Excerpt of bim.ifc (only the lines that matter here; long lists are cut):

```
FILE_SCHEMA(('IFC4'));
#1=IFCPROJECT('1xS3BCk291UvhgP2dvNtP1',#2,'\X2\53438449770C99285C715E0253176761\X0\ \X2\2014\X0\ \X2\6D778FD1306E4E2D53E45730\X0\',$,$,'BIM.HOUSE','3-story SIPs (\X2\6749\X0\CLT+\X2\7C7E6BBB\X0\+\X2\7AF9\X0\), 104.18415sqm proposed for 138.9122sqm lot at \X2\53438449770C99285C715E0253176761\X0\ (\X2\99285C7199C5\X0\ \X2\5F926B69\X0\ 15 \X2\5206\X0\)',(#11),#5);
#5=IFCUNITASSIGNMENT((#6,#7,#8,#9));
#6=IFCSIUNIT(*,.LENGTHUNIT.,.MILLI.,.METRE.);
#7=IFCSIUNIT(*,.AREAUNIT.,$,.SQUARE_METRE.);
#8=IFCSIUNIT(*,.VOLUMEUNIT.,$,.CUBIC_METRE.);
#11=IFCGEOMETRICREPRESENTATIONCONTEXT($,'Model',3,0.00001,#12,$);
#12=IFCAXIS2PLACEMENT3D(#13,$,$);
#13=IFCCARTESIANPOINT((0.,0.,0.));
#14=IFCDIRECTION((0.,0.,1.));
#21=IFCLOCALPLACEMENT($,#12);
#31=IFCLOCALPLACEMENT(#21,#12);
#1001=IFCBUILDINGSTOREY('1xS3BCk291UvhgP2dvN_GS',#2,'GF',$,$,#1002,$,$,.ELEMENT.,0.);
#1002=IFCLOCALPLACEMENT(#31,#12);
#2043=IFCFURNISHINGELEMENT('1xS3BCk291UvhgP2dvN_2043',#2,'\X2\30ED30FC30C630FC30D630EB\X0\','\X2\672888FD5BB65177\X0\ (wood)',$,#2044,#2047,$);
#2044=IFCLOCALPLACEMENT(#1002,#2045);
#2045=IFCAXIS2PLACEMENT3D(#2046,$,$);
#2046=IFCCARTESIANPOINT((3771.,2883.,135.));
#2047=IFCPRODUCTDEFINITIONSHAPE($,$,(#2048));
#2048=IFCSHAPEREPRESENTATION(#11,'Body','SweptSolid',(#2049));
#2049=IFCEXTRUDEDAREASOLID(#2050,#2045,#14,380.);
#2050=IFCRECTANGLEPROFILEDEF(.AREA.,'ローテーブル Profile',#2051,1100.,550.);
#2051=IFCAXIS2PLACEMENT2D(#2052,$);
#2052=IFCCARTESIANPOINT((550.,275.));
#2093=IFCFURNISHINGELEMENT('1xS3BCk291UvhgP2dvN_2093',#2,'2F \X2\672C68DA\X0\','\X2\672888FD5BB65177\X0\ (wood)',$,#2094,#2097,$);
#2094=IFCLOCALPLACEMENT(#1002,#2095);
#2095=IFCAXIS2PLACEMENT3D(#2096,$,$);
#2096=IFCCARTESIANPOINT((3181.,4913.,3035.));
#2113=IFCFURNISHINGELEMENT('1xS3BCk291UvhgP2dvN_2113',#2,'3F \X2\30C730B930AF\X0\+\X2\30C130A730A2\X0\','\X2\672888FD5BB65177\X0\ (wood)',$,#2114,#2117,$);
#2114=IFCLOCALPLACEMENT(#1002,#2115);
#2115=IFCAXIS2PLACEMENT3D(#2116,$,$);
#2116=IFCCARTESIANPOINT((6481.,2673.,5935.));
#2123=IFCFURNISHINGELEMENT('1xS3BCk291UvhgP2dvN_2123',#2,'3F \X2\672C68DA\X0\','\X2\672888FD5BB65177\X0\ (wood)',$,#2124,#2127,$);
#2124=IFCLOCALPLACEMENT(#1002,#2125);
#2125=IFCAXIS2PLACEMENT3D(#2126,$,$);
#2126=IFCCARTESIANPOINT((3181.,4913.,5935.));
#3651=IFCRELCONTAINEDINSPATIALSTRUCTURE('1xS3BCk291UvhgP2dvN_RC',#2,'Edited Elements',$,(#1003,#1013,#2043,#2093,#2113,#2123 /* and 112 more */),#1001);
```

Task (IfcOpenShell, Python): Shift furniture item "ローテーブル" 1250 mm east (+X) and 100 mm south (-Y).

```python
import ifcopenshell
import ifcopenshell.api.geometry
import ifcopenshell.util.placement
import ifcopenshell.util.unit

model = ifcopenshell.open("bim.ifc")
unit_scale = ifcopenshell.util.unit.calculate_unit_scale(model)

item = model.by_id(2043)
matrix = ifcopenshell.util.placement.get_local_placement(item.ObjectPlacement)
matrix[0, 3] += 1.25 / unit_scale
matrix[1, 3] -= 0.1 / unit_scale
ifcopenshell.api.geometry.edit_object_placement(model, product=item, matrix=matrix, is_si=False)

print(ifcopenshell.util.placement.get_local_placement(item.ObjectPlacement).round(3) + 0.0)

model.write("bim-out.ifc")
```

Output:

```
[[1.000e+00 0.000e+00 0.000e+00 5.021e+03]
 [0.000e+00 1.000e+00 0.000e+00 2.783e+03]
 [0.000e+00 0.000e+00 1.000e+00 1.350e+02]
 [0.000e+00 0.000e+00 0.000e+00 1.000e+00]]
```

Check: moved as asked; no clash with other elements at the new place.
